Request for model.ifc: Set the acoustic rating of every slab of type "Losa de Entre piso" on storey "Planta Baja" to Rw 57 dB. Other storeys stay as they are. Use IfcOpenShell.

First a look at what the model holds.

```python
import ifcopenshell
import ifcopenshell.util.element

model = ifcopenshell.open("model.ifc")
print(model.schema)
storey = next(s for s in model.by_type("IfcBuildingStorey") if s.Name == "Planta Baja")
slabs = [e for e in ifcopenshell.util.element.get_decomposition(storey) if e.is_a("IfcSlab")]
seen = {}
for e in slabs:
    element_type = ifcopenshell.util.element.get_type(e)
    key = (element_type.Name if element_type != e and element_type else None, ifcopenshell.util.element.get_pset(e, "Pset_SlabCommon", "AcousticRating"))
    seen[key] = seen.get(key, 0) + 1
for (name, value), count in sorted(seen.items(), key=str):
    print(count, "x", name, "|", value)
```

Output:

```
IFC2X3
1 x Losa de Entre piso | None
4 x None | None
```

```python
import ifcopenshell
import ifcopenshell.api.pset
import ifcopenshell.util.element

model = ifcopenshell.open("model.ifc")

storey = next(s for s in model.by_type("IfcBuildingStorey") if s.Name == "Planta Baja")
slabs = [e for e in ifcopenshell.util.element.get_decomposition(storey) if e.is_a("IfcSlab")]

count = 0
for e in slabs:
    element_type = ifcopenshell.util.element.get_type(e)
    if element_type in (None, e) or element_type.Name != "Losa de Entre piso":
        continue
    # add_pset returns the element's existing set when there is one.
    pset = ifcopenshell.api.pset.add_pset(model, product=e, name="Pset_SlabCommon")
    ifcopenshell.api.pset.edit_pset(model, pset=pset, properties={"AcousticRating": "Rw 57 dB"})
    count += 1

print(count, "slabs updated")

model.write("model_updated.ifc")
```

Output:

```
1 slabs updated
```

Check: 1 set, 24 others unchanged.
